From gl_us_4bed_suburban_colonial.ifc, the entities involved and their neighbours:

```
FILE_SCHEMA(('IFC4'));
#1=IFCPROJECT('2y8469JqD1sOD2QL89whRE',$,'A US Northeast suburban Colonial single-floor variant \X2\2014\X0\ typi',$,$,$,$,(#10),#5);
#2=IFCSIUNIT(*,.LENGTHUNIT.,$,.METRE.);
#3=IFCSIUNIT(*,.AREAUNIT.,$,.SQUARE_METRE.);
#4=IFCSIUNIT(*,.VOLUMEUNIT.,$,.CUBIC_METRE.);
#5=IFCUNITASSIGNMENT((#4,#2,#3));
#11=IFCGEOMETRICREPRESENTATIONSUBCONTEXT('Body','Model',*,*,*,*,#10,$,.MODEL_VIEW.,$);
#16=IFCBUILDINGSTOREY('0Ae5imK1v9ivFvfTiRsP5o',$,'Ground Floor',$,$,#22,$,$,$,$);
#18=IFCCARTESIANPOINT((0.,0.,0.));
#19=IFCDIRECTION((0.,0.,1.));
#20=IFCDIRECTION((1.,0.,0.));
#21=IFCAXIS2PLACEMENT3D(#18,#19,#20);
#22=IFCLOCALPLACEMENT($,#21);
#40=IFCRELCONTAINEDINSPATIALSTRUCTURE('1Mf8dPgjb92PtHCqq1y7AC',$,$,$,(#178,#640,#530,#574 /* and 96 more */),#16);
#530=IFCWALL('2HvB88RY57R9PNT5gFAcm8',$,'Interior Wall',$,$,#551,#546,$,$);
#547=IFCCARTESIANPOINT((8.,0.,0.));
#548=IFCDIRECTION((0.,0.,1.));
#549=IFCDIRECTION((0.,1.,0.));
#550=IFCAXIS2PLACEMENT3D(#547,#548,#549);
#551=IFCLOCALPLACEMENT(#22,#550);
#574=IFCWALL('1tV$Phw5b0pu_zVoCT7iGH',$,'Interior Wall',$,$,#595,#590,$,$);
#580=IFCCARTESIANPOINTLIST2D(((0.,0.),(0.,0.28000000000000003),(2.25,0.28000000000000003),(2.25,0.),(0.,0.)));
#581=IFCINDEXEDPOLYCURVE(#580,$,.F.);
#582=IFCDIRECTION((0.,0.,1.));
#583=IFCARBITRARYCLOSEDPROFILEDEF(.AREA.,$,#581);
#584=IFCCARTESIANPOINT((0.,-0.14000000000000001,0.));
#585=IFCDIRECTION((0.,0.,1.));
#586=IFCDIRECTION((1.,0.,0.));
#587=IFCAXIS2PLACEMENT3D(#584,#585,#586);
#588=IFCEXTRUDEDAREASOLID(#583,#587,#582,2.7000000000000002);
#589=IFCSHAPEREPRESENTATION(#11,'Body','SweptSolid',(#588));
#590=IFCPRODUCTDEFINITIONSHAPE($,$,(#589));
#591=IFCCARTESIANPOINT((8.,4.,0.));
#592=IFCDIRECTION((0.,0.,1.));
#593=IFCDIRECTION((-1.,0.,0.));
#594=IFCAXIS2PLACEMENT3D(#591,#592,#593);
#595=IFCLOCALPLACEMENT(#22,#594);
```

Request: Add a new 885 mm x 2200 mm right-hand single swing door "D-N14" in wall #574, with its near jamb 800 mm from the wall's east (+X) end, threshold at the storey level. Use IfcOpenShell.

```python
import numpy as np
import ifcopenshell
import ifcopenshell.api.feature
import ifcopenshell.api.geometry
import ifcopenshell.api.root
import ifcopenshell.api.spatial
import ifcopenshell.geom
import ifcopenshell.util.element
import ifcopenshell.util.placement
import ifcopenshell.util.representation
import ifcopenshell.util.shape
import ifcopenshell.util.unit

model = ifcopenshell.open("gl_us_4bed_suburban_colonial.ifc")
unit_scale = ifcopenshell.util.unit.calculate_unit_scale(model)
settings = ifcopenshell.geom.settings()


def volume(element):
    """Net volume in cubic metres, openings subtracted."""
    shape = ifcopenshell.geom.create_shape(settings, element)
    return ifcopenshell.util.shape.get_volume(shape.geometry)


wall = model.by_guid("1tV$Phw5b0pu_zVoCT7iGH")
storey = ifcopenshell.util.element.get_container(wall, ifc_class="IfcBuildingStorey")
context = ifcopenshell.util.representation.get_context(model, "Model", "Body", "MODEL_VIEW")
before = volume(wall)

width, height, from_end, sill = 0.885, 2.2, 0.8, 0.0  # metres

# The wall runs along its own X axis, and the end named is its -X end.
wall_shape = ifcopenshell.geom.create_shape(settings, wall)
x, y, z = ifcopenshell.util.shape.get_vertices(wall_shape.geometry).T
start = x.min() + from_end
face, thickness = float(y.min()), float(y.max() - y.min())
wall_matrix = ifcopenshell.util.placement.get_local_placement(wall.ObjectPlacement)
level = ifcopenshell.util.placement.get_local_placement(storey.ObjectPlacement)[2, 3]


def in_wall(x, y):
    """Placement at x, y metres in the wall's axes, at sill height."""
    matrix = wall_matrix.copy()
    matrix[:, 3] = wall_matrix @ np.array([x / unit_scale, y / unit_scale, 0.0, 1.0])
    matrix[2, 3] = level + sill / unit_scale
    return matrix


# Opening: a box that overshoots both wall faces by 50 mm.
opening = ifcopenshell.api.root.create_entity(model, ifc_class="IfcOpeningElement", predefined_type="OPENING")
box = ifcopenshell.api.geometry.add_wall_representation(
    model, context=context, length=width, height=height, thickness=thickness + 0.1
)
ifcopenshell.api.geometry.assign_representation(model, product=opening, representation=box)
ifcopenshell.api.geometry.edit_object_placement(model, product=opening, matrix=in_wall(start, face - 0.05), is_si=False)
ifcopenshell.api.feature.add_feature(model, feature=opening, element=wall)

door = ifcopenshell.api.root.create_entity(model, ifc_class="IfcDoor", name="D-N14", predefined_type="DOOR")
door.OverallWidth, door.OverallHeight = width / unit_scale, height / unit_scale
door.OperationType = "SINGLE_SWING_RIGHT"
body = ifcopenshell.api.geometry.add_door_representation(
    model,
    context=context,
    overall_width=door.OverallWidth,
    overall_height=door.OverallHeight,
    operation_type="SINGLE_SWING_RIGHT",
    lining_properties={"LiningDepth": thickness / unit_scale, "ThresholdDepth": thickness / unit_scale},
)
ifcopenshell.api.geometry.assign_representation(model, product=door, representation=body)
ifcopenshell.api.spatial.assign_container(model, products=[door], relating_structure=storey)
ifcopenshell.api.feature.add_filling(model, opening=opening, element=door)

# The lining spans the wall, so the door starts at the wall face.
ifcopenshell.api.geometry.edit_object_placement(model, product=door, matrix=in_wall(start, face), is_si=False)

after = volume(wall)

print(f"wall volume {before:.3f} -> {after:.3f} m3")

model.write("gl_us_4bed_suburban_colonial_rev.ifc")
```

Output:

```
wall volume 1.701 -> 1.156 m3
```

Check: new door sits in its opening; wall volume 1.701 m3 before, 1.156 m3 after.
